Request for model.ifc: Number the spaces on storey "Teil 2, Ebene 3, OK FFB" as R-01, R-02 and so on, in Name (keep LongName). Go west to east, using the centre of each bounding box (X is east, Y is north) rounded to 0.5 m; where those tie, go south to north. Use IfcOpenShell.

First a look at what the model holds.

```python
import ifcopenshell
import ifcopenshell.util.element
import ifcopenshell.util.placement

model = ifcopenshell.open("model.ifc")
print(model.schema)
storey = next(s for s in model.by_type("IfcBuildingStorey") if s.Name == "Teil 2, Ebene 3, OK FFB")
spaces = [e for e in ifcopenshell.util.element.get_decomposition(storey) if e.is_a("IfcSpace")]
for e in sorted(spaces, key=lambda e: e.id()):
    origin = ifcopenshell.util.placement.get_local_placement(e.ObjectPlacement)[:3, 3]
    print(e.id(), e.Name, e.LongName, origin.round(2) + 0.0, sep=" | ")
```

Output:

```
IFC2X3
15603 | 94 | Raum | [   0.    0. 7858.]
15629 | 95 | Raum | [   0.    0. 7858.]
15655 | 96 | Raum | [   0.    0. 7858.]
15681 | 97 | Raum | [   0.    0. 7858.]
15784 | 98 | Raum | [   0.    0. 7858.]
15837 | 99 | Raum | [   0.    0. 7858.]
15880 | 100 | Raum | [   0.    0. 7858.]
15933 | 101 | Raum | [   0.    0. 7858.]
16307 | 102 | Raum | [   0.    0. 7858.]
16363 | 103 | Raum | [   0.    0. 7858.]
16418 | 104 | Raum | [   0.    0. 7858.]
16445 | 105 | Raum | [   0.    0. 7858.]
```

```python
import ifcopenshell
import ifcopenshell.geom
import ifcopenshell.util.element
import ifcopenshell.util.shape

model = ifcopenshell.open("model.ifc")
settings = ifcopenshell.geom.settings()
settings.set("use-world-coords", True)


def centre(element):
    shape = ifcopenshell.geom.create_shape(settings, element)
    return ifcopenshell.util.shape.get_bbox_centroid(shape.geometry)


storey = next(s for s in model.by_type("IfcBuildingStorey") if s.Name == "Teil 2, Ebene 3, OK FFB")
spaces = [e for e in ifcopenshell.util.element.get_decomposition(storey) if e.is_a("IfcSpace")]

# Insertion points can sit at a corner or the storey origin, so sort by the geometry (in metres).
centres = {e: centre(e) for e in spaces}
spaces.sort(key=lambda e: (round(centres[e][0] / 0.5), centres[e][1]))

for i, e in enumerate(spaces, start=1):
    number = f"R-{i:02d}"
    e.Name = number
    print(e.id(), number)

model.write("model-out.ifc")
```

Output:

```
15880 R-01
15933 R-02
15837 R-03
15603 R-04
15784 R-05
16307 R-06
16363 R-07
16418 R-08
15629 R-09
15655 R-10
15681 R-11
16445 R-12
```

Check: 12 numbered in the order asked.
